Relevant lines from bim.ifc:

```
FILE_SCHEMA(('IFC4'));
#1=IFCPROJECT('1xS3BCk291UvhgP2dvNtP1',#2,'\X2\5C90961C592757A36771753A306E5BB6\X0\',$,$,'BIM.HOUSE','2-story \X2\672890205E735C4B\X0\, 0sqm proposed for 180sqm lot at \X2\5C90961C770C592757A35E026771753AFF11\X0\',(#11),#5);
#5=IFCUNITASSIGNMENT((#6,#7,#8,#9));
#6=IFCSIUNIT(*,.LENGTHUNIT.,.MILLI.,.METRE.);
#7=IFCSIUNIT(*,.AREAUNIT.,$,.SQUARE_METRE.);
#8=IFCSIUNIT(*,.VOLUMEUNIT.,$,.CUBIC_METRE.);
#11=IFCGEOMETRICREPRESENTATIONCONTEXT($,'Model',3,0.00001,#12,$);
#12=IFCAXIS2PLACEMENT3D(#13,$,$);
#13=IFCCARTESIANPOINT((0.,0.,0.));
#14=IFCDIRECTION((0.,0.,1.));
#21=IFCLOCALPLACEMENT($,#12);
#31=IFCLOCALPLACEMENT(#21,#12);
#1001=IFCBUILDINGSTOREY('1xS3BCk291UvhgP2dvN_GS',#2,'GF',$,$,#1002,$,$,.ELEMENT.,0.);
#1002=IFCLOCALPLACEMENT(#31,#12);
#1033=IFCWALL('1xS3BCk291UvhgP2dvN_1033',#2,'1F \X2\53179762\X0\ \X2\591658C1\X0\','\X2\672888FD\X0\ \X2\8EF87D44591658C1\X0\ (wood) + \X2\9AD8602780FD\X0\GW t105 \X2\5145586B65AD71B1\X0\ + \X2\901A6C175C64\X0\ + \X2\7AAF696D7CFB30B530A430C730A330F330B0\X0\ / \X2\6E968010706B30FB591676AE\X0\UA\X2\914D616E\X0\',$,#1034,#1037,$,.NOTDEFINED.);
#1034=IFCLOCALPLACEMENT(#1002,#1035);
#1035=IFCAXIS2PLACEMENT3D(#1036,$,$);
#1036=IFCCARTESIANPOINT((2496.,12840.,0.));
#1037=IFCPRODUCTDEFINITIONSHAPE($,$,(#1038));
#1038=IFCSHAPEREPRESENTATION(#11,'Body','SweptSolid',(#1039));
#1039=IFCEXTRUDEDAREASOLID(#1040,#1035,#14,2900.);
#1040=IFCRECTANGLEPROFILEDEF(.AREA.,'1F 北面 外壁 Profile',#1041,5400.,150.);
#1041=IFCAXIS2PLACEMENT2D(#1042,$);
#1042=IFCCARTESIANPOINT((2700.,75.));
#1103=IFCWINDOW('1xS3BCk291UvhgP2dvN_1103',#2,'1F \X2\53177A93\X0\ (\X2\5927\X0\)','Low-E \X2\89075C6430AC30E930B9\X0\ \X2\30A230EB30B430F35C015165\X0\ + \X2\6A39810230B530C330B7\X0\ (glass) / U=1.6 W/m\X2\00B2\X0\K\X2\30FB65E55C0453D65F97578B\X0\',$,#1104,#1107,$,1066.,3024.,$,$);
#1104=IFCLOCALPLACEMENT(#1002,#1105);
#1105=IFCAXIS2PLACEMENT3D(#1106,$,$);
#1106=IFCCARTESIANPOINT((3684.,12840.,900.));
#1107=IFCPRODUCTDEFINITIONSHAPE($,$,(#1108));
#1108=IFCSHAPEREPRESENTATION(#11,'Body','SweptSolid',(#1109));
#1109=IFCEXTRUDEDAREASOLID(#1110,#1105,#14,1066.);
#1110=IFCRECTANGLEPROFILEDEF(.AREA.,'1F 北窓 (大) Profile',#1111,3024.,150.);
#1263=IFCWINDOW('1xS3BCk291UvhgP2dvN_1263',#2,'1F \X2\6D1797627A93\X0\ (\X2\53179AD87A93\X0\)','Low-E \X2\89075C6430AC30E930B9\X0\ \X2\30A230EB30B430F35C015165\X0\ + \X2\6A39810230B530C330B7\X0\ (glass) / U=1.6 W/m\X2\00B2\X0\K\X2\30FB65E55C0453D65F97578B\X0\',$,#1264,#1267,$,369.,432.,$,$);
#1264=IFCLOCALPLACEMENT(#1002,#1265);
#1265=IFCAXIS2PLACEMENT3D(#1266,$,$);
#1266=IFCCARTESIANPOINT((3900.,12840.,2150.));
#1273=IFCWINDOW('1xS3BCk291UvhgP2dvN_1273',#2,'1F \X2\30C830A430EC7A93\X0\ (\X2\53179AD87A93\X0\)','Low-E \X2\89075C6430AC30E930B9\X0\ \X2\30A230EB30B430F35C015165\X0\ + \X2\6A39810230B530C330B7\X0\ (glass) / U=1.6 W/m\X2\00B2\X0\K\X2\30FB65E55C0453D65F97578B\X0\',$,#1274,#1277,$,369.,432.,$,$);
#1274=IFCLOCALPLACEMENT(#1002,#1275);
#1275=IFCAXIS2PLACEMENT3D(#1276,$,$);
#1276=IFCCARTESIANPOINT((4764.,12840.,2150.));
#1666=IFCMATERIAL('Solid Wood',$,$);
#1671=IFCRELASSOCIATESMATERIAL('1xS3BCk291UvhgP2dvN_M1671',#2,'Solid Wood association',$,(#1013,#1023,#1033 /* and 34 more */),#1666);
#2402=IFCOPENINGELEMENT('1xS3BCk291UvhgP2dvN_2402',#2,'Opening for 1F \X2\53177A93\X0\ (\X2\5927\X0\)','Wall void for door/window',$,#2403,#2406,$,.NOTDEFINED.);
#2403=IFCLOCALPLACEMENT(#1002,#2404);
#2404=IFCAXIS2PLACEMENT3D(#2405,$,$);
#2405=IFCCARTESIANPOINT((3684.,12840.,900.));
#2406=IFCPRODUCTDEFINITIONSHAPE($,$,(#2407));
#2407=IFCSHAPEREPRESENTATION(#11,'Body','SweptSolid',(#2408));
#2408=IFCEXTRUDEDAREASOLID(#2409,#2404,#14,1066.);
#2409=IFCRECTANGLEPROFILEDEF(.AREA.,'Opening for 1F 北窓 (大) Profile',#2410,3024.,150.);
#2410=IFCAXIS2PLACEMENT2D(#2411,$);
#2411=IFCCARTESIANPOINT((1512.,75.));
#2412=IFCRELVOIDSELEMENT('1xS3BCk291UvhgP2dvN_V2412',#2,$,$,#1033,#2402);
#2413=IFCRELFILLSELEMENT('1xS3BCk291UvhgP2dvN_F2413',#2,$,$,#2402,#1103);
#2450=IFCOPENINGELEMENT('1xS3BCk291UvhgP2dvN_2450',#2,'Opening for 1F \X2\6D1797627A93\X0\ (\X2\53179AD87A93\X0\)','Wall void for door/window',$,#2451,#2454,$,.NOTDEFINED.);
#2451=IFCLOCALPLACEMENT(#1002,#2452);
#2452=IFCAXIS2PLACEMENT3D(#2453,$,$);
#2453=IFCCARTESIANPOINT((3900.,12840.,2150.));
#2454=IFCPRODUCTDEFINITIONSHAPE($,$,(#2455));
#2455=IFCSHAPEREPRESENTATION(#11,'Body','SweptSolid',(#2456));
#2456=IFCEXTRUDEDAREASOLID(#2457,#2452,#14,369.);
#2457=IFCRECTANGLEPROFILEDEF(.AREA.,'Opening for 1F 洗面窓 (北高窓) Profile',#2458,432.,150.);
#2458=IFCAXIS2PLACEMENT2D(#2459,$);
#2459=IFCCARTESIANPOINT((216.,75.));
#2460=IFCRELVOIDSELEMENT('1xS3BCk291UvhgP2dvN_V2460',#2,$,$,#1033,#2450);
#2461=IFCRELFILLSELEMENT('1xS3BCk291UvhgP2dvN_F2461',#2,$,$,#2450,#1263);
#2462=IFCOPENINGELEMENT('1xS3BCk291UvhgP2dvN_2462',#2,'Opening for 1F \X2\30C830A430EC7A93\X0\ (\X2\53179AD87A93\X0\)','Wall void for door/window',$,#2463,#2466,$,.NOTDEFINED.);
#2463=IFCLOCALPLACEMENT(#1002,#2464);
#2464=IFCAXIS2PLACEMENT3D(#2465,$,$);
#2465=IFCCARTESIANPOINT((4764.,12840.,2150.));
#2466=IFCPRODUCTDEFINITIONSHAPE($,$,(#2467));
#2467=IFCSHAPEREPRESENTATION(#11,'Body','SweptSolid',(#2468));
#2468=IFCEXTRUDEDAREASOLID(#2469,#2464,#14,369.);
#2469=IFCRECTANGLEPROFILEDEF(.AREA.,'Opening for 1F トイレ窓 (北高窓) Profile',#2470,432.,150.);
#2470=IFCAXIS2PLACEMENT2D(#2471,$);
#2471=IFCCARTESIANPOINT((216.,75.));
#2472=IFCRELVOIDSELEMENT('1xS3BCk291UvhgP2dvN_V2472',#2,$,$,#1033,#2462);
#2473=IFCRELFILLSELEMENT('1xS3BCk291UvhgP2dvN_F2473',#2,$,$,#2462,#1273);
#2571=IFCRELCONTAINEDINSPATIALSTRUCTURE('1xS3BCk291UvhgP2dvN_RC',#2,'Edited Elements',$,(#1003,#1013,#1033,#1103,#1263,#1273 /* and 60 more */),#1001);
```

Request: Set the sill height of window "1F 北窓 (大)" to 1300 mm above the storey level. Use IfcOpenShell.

```python
import numpy as np
import ifcopenshell
import ifcopenshell.api.geometry
import ifcopenshell.geom
import ifcopenshell.util.element
import ifcopenshell.util.placement
import ifcopenshell.util.shape
import ifcopenshell.util.unit

model = ifcopenshell.open("bim.ifc")
unit_scale = ifcopenshell.util.unit.calculate_unit_scale(model)

window = model.by_id(1103)
opening = window.FillsVoids[0].RelatingOpeningElement
storey = ifcopenshell.util.element.get_container(window, ifc_class="IfcBuildingStorey")
level = ifcopenshell.util.placement.get_local_placement(storey.ObjectPlacement)[2, 3]

# The opening's origin need not be at the sill, so measure its lowest point.
shape = ifcopenshell.geom.create_shape(ifcopenshell.geom.settings(), opening)
bottom = ifcopenshell.util.shape.get_shape_bottom_elevation(shape, shape.geometry) / unit_scale
dz = level + 1.3 / unit_scale - bottom

shift = np.array([0.0, 0.0, dz])
# The window is not placed relative to its opening, so move both.
for product in (opening, window):
    matrix = ifcopenshell.util.placement.get_local_placement(product.ObjectPlacement)
    matrix[:3, 3] += shift
    ifcopenshell.api.geometry.edit_object_placement(model, product=product, matrix=matrix, is_si=False)

print(f"moved by {dz * unit_scale:+.3f} m")

model.write("bim_v2.ifc")
```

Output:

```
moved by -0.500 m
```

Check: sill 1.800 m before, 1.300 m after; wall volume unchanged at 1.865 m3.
